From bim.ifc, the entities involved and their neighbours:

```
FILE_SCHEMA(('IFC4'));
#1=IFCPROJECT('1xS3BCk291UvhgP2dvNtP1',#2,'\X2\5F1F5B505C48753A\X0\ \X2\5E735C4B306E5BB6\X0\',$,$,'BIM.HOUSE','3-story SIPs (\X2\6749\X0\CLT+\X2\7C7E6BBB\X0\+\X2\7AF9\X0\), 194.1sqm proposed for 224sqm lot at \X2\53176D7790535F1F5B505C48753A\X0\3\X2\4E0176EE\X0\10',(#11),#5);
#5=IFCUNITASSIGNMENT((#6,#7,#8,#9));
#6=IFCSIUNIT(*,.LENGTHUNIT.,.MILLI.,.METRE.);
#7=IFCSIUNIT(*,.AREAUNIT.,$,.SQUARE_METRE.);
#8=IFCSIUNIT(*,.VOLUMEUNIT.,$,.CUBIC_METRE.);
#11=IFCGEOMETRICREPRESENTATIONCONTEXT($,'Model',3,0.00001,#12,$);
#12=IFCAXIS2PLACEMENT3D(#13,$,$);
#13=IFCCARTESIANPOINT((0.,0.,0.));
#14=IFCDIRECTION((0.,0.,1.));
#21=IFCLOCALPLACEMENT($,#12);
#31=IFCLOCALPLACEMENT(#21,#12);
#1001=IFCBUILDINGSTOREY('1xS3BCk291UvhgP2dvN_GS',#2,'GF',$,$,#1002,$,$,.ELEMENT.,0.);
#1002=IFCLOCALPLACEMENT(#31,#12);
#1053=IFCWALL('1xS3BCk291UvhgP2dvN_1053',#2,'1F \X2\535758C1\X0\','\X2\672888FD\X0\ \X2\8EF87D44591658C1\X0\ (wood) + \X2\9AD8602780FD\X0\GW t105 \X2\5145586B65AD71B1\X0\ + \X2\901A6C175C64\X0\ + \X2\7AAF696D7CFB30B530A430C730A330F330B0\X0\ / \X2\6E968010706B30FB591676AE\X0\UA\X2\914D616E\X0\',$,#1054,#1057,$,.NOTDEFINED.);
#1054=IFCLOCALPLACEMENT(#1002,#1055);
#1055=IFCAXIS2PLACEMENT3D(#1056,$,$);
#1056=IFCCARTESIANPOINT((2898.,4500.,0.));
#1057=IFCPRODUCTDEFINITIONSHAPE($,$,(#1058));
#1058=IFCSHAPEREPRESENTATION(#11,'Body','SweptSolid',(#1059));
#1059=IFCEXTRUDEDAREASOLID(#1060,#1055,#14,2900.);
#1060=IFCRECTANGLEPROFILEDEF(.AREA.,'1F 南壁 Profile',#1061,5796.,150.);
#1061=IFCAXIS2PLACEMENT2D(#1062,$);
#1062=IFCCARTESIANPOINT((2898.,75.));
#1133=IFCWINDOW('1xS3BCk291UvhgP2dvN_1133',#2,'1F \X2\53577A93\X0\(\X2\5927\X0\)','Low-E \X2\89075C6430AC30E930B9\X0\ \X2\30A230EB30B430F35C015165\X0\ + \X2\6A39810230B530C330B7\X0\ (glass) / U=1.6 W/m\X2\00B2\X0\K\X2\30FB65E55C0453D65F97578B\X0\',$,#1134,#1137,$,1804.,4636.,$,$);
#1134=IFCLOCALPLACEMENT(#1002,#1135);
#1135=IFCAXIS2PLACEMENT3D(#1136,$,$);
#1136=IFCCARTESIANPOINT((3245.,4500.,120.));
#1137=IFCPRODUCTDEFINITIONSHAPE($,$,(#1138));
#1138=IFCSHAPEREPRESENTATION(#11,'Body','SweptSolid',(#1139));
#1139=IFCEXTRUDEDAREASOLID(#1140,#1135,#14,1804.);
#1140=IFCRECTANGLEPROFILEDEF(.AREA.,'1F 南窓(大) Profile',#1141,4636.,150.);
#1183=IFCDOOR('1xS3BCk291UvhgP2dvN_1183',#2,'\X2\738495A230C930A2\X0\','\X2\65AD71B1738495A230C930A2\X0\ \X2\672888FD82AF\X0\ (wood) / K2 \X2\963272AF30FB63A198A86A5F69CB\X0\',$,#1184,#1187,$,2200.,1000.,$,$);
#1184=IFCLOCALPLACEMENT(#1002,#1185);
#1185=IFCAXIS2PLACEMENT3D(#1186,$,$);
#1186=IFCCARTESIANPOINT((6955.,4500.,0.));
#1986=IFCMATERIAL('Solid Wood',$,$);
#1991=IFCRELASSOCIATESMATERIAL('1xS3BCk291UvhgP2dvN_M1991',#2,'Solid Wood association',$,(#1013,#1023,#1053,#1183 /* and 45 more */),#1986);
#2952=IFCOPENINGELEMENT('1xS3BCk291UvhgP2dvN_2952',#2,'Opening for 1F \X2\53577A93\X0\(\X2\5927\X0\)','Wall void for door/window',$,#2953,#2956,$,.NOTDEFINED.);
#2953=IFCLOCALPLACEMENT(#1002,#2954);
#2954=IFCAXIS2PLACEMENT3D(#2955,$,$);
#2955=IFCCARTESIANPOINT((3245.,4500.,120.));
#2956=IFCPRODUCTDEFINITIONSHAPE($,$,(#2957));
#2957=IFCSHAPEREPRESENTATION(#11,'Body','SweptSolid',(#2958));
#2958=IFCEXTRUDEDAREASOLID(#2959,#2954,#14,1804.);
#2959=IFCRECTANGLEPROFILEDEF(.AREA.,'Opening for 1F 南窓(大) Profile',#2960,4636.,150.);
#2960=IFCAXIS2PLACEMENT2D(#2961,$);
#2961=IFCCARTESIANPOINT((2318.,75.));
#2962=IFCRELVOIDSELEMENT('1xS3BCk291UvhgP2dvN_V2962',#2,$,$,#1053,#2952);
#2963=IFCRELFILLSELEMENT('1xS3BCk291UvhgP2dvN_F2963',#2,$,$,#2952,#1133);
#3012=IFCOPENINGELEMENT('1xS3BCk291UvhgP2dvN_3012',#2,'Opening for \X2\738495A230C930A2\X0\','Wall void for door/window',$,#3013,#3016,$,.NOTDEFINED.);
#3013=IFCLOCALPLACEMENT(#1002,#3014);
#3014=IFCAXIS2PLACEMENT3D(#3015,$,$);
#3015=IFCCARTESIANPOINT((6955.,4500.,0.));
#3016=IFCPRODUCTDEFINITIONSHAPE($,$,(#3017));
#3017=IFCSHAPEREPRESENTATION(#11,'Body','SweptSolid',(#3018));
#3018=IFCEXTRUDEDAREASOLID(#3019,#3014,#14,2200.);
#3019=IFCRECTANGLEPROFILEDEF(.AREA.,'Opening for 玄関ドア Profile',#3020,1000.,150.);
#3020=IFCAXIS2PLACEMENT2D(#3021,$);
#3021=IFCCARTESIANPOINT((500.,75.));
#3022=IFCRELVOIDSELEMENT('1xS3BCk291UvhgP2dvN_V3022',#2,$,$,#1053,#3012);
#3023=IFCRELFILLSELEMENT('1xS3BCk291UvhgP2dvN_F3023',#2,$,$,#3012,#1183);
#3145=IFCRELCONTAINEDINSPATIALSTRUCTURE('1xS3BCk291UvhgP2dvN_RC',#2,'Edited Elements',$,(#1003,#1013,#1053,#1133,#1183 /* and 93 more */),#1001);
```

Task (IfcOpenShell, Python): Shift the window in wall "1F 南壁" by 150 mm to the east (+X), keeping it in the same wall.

```python
import ifcopenshell
import ifcopenshell.api.geometry
import ifcopenshell.util.placement
import ifcopenshell.util.unit

model = ifcopenshell.open("bim.ifc")
unit_scale = ifcopenshell.util.unit.calculate_unit_scale(model)

window = model.by_id(1133)
opening = window.FillsVoids[0].RelatingOpeningElement
wall = opening.VoidsElements[0].RelatingBuildingElement

wall_matrix = ifcopenshell.util.placement.get_local_placement(wall.ObjectPlacement)
shift = wall_matrix[:3, 0] * 0.15 / unit_scale
before = ifcopenshell.util.placement.get_local_placement(window.ObjectPlacement)[:3, 3].copy()

# The window is not placed relative to its opening, so move both.
for product in (opening, window):
    matrix = ifcopenshell.util.placement.get_local_placement(product.ObjectPlacement)
    matrix[:3, 3] += shift
    ifcopenshell.api.geometry.edit_object_placement(model, product=product, matrix=matrix, is_si=False)

after = ifcopenshell.util.placement.get_local_placement(window.ObjectPlacement)[:3, 3]
print("window moved by", (after - before).round(3) + 0.0)

model.write("bim_edited.ifc")
```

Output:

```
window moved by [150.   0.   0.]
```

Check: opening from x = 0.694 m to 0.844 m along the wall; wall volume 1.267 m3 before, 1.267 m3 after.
